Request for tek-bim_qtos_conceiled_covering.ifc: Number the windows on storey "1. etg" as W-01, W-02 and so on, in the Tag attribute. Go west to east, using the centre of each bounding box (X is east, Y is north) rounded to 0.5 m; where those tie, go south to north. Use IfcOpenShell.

First a look at what the model holds.

```python
import ifcopenshell
import ifcopenshell.util.element
import ifcopenshell.util.placement

model = ifcopenshell.open("tek-bim_qtos_conceiled_covering.ifc")
print(model.schema)
storey = next(s for s in model.by_type("IfcBuildingStorey") if s.Name == "1. etg")
windows = [e for e in ifcopenshell.util.element.get_decomposition(storey) if e.is_a("IfcWindow")]
for e in sorted(windows, key=lambda e: e.id()):
    origin = ifcopenshell.util.placement.get_local_placement(e.ObjectPlacement)[:3, 3]
    print(e.id(), e.Tag, e.Name, origin.round(2) + 0.0, sep=" | ")
```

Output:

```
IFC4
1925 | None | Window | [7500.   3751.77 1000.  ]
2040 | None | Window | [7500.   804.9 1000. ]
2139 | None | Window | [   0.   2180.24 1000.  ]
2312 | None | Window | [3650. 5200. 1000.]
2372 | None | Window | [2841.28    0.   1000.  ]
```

```python
import ifcopenshell
import ifcopenshell.geom
import ifcopenshell.util.element
import ifcopenshell.util.shape

model = ifcopenshell.open("tek-bim_qtos_conceiled_covering.ifc")
settings = ifcopenshell.geom.settings()
settings.set("use-world-coords", True)


def centre(element):
    shape = ifcopenshell.geom.create_shape(settings, element)
    return ifcopenshell.util.shape.get_bbox_centroid(shape.geometry)


storey = next(s for s in model.by_type("IfcBuildingStorey") if s.Name == "1. etg")
windows = [e for e in ifcopenshell.util.element.get_decomposition(storey) if e.is_a("IfcWindow")]

# Insertion points can sit at a corner or the storey origin, so sort by the geometry (in metres).
centres = {e: centre(e) for e in windows}
windows.sort(key=lambda e: (round(centres[e][0] / 0.5), centres[e][1]))

for i, e in enumerate(windows, start=1):
    number = f"W-{i:02d}"
    e.Tag = number
    print(e.id(), number)

model.write("tek-bim_qtos_conceiled_covering_rev.ifc")
```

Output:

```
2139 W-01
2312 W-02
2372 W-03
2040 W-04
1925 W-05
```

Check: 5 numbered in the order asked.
